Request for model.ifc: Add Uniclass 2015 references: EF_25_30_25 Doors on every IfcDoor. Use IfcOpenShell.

First a look at what the model holds.

```python
import ifcopenshell

model = ifcopenshell.open("model.ifc")
print(model.schema)
print("classifications:", [c.Name for c in model.by_type("IfcClassification")])
for ifc_class in ("IfcDoor", "IfcRoof", "IfcStair", "IfcWall", "IfcWindow"):
    print(ifc_class, len(model.by_type(ifc_class)))
```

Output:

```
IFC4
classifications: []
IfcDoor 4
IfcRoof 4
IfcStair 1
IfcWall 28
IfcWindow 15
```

```python
import ifcopenshell
import ifcopenshell.api.classification

model = ifcopenshell.open("model.ifc")

system = ifcopenshell.api.classification.add_classification(model, classification="Uniclass 2015")

codes = {
    "IfcDoor": ("EF_25_30_25", "Doors"),
}
for ifc_class, (code, name) in codes.items():
    products = model.by_type(ifc_class)
    ifcopenshell.api.classification.add_reference(
        model, products=products, classification=system, identification=code, name=name
    )
    print(code, len(products))

model.write("model_v2.ifc")
```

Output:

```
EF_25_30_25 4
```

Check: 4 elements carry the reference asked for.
